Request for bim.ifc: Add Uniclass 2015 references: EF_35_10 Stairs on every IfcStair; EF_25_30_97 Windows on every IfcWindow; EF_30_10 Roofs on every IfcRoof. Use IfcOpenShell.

First a look at what the model holds.

```python
import ifcopenshell

model = ifcopenshell.open("bim.ifc")
print(model.schema)
print("classifications:", [c.Name for c in model.by_type("IfcClassification")])
for ifc_class in ("IfcDoor", "IfcRoof", "IfcStair", "IfcWall", "IfcWindow"):
    print(ifc_class, len(model.by_type(ifc_class)))
```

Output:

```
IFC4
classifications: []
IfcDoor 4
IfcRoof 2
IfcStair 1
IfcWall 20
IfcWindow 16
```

```python
import ifcopenshell
import ifcopenshell.api.classification

model = ifcopenshell.open("bim.ifc")

system = ifcopenshell.api.classification.add_classification(model, classification="Uniclass 2015")

codes = {
    "IfcStair": ("EF_35_10", "Stairs"),
    "IfcWindow": ("EF_25_30_97", "Windows"),
    "IfcRoof": ("EF_30_10", "Roofs"),
}
for ifc_class, (code, name) in codes.items():
    products = model.by_type(ifc_class)
    ifcopenshell.api.classification.add_reference(
        model, products=products, classification=system, identification=code, name=name
    )
    print(code, len(products))

model.write("bim_edited.ifc")
```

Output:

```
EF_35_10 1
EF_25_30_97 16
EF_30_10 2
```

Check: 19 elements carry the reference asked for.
